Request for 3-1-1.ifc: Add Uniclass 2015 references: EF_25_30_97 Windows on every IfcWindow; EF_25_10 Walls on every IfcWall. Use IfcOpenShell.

First a look at what the model holds.

```python
import ifcopenshell

model = ifcopenshell.open("3-1-1.ifc")
print(model.schema)
print("classifications:", [c.Name for c in model.by_type("IfcClassification")])
for ifc_class in ("IfcDoor", "IfcRoof", "IfcStair", "IfcWall", "IfcWindow"):
    print(ifc_class, len(model.by_type(ifc_class)))
```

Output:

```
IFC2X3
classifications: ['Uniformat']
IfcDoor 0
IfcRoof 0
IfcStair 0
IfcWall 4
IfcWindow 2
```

```python
import ifcopenshell
import ifcopenshell.api.classification

model = ifcopenshell.open("3-1-1.ifc")

# IFC2X3 requires Source and Edition and has no link from the project to the system.
system = model.create_entity("IfcClassification", Source="NBS", Edition="2015", Name="Uniclass 2015")

codes = {
    "IfcWindow": ("EF_25_30_97", "Windows"),
    "IfcWall": ("EF_25_10", "Walls"),
}
for ifc_class, (code, name) in codes.items():
    products = model.by_type(ifc_class)
    ifcopenshell.api.classification.add_reference(
        model, products=products, classification=system, identification=code, name=name
    )
    print(code, len(products))

model.write("3-1-1_v2.ifc")
```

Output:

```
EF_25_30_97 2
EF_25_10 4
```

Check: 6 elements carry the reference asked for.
